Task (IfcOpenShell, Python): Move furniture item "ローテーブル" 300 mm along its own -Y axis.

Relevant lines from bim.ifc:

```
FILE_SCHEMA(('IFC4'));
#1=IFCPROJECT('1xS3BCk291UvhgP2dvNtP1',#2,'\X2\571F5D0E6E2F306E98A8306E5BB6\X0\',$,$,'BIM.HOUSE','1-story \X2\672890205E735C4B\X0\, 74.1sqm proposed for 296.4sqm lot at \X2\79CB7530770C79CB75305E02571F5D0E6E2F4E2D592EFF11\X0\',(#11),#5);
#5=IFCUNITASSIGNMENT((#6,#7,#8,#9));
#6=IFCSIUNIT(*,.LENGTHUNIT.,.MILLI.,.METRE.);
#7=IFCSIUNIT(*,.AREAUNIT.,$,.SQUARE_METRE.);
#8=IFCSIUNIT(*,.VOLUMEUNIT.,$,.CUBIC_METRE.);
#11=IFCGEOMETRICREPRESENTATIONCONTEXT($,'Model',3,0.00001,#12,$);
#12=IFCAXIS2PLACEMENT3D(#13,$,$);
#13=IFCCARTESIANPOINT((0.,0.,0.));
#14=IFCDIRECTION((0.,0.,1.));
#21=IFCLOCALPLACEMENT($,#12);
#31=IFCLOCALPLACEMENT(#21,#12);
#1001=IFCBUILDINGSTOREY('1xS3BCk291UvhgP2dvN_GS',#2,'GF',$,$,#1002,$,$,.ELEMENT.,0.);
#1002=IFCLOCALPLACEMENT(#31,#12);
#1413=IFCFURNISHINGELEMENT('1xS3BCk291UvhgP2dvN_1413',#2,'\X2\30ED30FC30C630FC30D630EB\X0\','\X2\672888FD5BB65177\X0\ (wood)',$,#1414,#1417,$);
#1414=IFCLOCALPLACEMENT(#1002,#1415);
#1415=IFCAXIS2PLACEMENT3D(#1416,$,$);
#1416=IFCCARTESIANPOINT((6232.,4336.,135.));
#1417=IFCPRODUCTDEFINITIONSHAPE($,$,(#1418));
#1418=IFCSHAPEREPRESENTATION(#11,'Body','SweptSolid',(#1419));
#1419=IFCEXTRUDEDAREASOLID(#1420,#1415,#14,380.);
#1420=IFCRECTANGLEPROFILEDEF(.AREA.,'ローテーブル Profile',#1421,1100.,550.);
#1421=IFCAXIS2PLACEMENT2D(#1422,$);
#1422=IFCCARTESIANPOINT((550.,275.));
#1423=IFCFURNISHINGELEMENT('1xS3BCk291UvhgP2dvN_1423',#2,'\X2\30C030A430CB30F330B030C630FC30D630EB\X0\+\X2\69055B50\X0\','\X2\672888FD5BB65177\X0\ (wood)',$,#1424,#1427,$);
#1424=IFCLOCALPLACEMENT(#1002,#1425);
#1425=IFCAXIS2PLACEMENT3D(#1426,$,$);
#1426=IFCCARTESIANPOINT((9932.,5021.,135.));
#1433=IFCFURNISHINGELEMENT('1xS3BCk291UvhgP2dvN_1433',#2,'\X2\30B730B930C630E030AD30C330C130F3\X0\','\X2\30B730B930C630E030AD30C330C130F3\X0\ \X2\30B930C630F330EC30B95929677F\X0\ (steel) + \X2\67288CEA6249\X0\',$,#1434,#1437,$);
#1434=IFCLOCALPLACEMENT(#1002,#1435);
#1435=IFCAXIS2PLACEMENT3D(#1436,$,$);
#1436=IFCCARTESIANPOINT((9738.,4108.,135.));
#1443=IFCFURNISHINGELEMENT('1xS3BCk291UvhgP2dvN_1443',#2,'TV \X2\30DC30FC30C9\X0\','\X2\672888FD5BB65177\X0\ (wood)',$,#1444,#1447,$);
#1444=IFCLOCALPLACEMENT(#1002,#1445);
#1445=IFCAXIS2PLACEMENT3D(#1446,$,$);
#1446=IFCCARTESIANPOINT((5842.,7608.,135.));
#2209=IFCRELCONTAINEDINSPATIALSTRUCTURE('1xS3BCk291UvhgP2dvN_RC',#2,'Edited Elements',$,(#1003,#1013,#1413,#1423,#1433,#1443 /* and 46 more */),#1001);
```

```python
import ifcopenshell
import ifcopenshell.api.geometry
import ifcopenshell.util.placement

model = ifcopenshell.open("bim.ifc")

item = model.by_id(1413)
matrix = ifcopenshell.util.placement.get_local_placement(item.ObjectPlacement)
matrix[:3, 3] -= matrix[:3, 1] * 300.0
ifcopenshell.api.geometry.edit_object_placement(model, product=item, matrix=matrix, is_si=False)

print(ifcopenshell.util.placement.get_local_placement(item.ObjectPlacement).round(3) + 0.0)

model.write("bim-out.ifc")
```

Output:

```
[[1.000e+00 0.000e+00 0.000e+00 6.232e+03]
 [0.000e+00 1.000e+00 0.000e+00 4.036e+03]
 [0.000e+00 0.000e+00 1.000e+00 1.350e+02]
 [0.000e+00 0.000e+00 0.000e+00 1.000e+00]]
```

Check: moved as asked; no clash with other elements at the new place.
